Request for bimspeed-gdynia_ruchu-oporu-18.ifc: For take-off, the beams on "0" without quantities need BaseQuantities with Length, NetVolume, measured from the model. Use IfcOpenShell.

First a look at what the model holds.

```python
import ifcopenshell
import ifcopenshell.util.element
import ifcopenshell.util.unit

model = ifcopenshell.open("bimspeed-gdynia_ruchu-oporu-18.ifc")
print(model.schema)
for unit_type in ("LENGTHUNIT", "AREAUNIT", "VOLUMEUNIT"):
    print(unit_type, ifcopenshell.util.unit.calculate_unit_scale(model, unit_type))
storey = next(s for s in model.by_type("IfcBuildingStorey") if s.Name == "0")
beams = [e for e in ifcopenshell.util.element.get_decomposition(storey) if e.is_a("IfcBeam")]
for e in sorted(beams, key=lambda e: e.id()):
    print(e.id(), e.is_a(), e.Name, list(ifcopenshell.util.element.get_psets(e, qtos_only=True)), sep=" | ")
```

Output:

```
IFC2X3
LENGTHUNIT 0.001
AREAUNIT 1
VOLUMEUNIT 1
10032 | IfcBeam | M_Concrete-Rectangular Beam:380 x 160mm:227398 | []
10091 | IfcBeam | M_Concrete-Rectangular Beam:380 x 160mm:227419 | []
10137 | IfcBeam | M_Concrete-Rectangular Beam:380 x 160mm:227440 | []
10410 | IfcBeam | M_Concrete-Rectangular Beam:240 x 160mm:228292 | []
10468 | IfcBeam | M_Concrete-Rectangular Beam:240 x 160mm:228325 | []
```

```python
import ifcopenshell
import ifcopenshell.api.pset
import ifcopenshell.geom
import ifcopenshell.util.element
import ifcopenshell.util.shape
import ifcopenshell.util.unit

model = ifcopenshell.open("bimspeed-gdynia_ruchu-oporu-18.ifc")
unit_scale = ifcopenshell.util.unit.calculate_unit_scale(model)
volume_scale = ifcopenshell.util.unit.calculate_unit_scale(model, "VOLUMEUNIT")
settings = ifcopenshell.geom.settings()

storey = next(s for s in model.by_type("IfcBuildingStorey") if s.Name == "0")
beams = [e for e in ifcopenshell.util.element.get_decomposition(storey) if e.is_a("IfcBeam")]

for e in sorted(beams, key=lambda e: e.id()):
    if ifcopenshell.util.element.get_psets(e, qtos_only=True, should_inherit=False):
        continue
    # Geometry comes back in metres, in the element's own axes.
    shape = ifcopenshell.geom.create_shape(settings, e)
    values = {
        "Length": ifcopenshell.util.shape.get_max_xyz(shape.geometry) / unit_scale,
        "NetVolume": ifcopenshell.util.shape.get_volume(shape.geometry) / volume_scale,
    }
    qto = ifcopenshell.api.pset.add_qto(model, product=e, name="BaseQuantities")
    ifcopenshell.api.pset.edit_qto(model, qto=qto, properties=values)
    print(e.id(), {k: round(v, 3) for k, v in values.items()})

model.write("bimspeed-gdynia_ruchu-oporu-18_v2.ifc")
```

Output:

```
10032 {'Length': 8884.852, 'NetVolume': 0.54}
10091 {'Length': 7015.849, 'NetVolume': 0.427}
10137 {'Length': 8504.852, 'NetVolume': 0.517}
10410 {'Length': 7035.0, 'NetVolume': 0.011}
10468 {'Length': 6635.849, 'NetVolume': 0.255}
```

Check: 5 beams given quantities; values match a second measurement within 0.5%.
